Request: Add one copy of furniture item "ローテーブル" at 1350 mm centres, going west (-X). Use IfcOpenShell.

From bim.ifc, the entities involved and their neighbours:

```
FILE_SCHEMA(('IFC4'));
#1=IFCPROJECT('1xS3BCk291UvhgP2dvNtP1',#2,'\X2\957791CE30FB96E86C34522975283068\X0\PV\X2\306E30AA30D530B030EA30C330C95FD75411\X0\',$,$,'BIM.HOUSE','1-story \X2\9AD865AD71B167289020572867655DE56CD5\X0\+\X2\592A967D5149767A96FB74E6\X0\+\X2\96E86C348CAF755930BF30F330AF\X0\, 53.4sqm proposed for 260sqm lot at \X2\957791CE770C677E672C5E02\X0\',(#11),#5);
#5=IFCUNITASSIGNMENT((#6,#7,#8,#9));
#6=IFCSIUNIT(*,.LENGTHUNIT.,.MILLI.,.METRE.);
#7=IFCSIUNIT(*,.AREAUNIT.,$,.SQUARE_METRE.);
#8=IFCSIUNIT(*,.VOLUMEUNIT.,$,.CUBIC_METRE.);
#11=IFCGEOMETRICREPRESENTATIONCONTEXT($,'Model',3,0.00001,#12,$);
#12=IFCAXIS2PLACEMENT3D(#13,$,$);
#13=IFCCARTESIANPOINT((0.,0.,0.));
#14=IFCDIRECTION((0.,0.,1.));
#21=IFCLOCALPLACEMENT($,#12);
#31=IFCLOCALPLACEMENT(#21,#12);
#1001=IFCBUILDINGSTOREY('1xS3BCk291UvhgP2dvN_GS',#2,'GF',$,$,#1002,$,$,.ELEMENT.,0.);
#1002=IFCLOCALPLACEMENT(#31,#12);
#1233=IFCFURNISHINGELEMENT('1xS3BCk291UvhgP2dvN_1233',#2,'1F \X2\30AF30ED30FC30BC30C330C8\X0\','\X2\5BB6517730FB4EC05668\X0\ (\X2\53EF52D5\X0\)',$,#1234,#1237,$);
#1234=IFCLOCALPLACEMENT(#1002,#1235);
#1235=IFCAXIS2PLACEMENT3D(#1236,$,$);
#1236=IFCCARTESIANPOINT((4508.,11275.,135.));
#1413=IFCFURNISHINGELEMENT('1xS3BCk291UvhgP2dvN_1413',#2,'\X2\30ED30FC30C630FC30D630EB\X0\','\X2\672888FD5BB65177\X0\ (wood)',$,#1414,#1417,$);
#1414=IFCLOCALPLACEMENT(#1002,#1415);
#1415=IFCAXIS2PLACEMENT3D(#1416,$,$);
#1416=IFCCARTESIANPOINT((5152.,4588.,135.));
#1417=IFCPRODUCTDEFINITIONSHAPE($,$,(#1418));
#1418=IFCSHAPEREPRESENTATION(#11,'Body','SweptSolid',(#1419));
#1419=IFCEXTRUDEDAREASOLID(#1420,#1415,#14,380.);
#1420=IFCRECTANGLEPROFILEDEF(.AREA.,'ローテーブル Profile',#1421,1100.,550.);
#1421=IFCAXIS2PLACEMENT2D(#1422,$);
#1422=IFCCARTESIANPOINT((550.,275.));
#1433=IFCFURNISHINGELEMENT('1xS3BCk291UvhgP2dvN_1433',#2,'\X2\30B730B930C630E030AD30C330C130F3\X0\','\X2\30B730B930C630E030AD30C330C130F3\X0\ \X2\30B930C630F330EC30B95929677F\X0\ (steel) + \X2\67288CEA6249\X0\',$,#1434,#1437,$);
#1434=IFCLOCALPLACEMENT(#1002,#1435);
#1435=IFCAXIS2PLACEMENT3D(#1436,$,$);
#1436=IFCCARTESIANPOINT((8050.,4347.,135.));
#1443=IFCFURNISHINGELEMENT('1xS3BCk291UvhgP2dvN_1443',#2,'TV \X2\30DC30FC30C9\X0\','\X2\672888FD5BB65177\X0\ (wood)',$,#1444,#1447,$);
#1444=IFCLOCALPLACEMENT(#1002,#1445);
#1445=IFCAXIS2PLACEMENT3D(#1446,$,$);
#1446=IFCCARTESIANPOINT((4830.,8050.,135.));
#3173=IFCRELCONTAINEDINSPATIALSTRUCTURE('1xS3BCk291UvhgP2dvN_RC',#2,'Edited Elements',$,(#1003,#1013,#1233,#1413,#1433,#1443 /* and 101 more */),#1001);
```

```python
import numpy as np
import ifcopenshell
import ifcopenshell.api.geometry
import ifcopenshell.api.root
import ifcopenshell.util.element
import ifcopenshell.util.placement
import ifcopenshell.util.unit

model = ifcopenshell.open("bim.ifc")
unit_scale = ifcopenshell.util.unit.calculate_unit_scale(model)


def reuse_history(source, copy):
    """copy_class also copies each property set's owner history, people and application; keep the originals."""
    for rel in copy.IsDefinedBy:
        if rel.is_a("IfcRelDefinesByProperties") and (history := rel.RelatingPropertyDefinition.OwnerHistory):
            rel.RelatingPropertyDefinition.OwnerHistory = source.OwnerHistory
            ifcopenshell.util.element.remove_deep2(model, history)


source = model.by_id(1413)
base = ifcopenshell.util.placement.get_local_placement(source.ObjectPlacement)
step = np.array([-1.0, 0.0, 0.0]) * 1.35 / unit_scale

for i in range(1, 2):
    copy = ifcopenshell.api.root.copy_class(model, product=source)
    copy.Representation = ifcopenshell.util.element.copy_deep(
        model, source.Representation, exclude=["IfcGeometricRepresentationContext", "IfcRepresentationMap"]
    )
    reuse_history(source, copy)
    matrix = base.copy()
    matrix[:3, 3] += i * step
    print("added at", matrix[:3, 3].round(3) + 0.0)
    ifcopenshell.api.geometry.edit_object_placement(model, product=copy, matrix=matrix, is_si=False)

model.write("bim_v2.ifc")
```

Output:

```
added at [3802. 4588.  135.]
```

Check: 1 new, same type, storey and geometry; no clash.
